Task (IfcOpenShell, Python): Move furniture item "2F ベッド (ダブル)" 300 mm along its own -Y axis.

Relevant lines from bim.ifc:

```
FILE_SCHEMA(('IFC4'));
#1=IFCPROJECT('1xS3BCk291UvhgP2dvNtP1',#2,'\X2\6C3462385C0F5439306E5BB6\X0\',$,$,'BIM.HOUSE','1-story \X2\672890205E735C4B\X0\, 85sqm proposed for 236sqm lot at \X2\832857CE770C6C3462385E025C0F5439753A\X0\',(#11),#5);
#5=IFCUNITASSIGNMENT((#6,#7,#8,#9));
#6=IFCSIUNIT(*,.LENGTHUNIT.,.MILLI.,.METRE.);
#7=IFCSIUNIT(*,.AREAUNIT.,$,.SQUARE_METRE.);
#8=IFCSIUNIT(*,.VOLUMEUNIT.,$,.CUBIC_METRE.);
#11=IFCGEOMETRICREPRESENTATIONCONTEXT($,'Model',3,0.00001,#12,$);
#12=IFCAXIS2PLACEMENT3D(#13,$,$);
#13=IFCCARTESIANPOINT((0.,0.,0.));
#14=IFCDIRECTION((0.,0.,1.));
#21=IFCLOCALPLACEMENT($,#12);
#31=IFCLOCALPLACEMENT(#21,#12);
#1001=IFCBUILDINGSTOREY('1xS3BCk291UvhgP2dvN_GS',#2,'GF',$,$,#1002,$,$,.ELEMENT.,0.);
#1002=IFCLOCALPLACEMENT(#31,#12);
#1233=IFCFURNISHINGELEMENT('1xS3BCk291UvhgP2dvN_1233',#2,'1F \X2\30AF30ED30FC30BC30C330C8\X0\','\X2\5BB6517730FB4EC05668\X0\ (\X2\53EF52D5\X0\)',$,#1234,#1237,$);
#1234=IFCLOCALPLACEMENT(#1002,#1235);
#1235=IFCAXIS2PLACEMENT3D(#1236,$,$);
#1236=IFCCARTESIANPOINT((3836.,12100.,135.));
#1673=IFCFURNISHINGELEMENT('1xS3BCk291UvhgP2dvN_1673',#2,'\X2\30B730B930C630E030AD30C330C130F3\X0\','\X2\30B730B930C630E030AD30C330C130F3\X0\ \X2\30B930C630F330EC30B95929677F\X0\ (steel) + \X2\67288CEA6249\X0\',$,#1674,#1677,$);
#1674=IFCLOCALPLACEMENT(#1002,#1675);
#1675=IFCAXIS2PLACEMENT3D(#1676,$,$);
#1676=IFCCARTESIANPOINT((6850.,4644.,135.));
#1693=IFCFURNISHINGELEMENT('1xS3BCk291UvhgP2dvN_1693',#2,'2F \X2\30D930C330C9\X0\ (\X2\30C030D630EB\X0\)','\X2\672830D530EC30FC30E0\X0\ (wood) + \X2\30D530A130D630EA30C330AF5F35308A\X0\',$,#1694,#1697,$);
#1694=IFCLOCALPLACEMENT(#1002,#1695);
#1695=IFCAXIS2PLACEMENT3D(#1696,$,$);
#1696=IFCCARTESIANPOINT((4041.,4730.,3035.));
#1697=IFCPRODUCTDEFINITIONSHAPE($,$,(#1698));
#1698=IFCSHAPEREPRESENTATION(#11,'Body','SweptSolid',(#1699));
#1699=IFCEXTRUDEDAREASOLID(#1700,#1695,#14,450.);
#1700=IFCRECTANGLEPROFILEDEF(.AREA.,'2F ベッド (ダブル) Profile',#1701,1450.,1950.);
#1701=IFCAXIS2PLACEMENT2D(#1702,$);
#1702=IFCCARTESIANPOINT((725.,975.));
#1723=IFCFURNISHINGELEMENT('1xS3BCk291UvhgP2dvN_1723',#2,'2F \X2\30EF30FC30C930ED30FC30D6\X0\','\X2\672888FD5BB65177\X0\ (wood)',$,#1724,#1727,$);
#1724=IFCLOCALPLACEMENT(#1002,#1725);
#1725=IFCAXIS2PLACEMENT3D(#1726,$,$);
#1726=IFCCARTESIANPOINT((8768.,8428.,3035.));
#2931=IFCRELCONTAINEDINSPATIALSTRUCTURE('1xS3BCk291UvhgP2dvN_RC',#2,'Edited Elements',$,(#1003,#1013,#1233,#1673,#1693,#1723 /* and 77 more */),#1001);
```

```python
import ifcopenshell
import ifcopenshell.api.geometry
import ifcopenshell.util.placement
import ifcopenshell.util.unit

model = ifcopenshell.open("bim.ifc")
unit_scale = ifcopenshell.util.unit.calculate_unit_scale(model)

item = model.by_id(1693)
matrix = ifcopenshell.util.placement.get_local_placement(item.ObjectPlacement)
matrix[:3, 3] -= matrix[:3, 1] * 0.3 / unit_scale
ifcopenshell.api.geometry.edit_object_placement(model, product=item, matrix=matrix, is_si=False)

print(ifcopenshell.util.placement.get_local_placement(item.ObjectPlacement).round(3) + 0.0)

model.write("bim_rev.ifc")
```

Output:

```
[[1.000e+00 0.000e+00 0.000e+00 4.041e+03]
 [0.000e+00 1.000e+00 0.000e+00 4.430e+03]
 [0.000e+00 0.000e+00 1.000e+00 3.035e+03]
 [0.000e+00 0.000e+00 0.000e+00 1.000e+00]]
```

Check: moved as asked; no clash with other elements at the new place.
